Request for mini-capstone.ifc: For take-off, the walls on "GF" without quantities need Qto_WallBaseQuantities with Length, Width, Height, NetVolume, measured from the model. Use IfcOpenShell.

First a look at what the model holds.

```python
import ifcopenshell
import ifcopenshell.util.element
import ifcopenshell.util.unit

model = ifcopenshell.open("mini-capstone.ifc")
print(model.schema)
for unit_type in ("LENGTHUNIT", "AREAUNIT", "VOLUMEUNIT"):
    print(unit_type, ifcopenshell.util.unit.calculate_unit_scale(model, unit_type))
storey = next(s for s in model.by_type("IfcBuildingStorey") if s.Name == "GF")
walls = [e for e in ifcopenshell.util.element.get_decomposition(storey) if e.is_a("IfcWall")]
for e in sorted(walls, key=lambda e: e.id()):
    print(e.id(), e.is_a(), e.Name, list(ifcopenshell.util.element.get_psets(e, qtos_only=True)), sep=" | ")
```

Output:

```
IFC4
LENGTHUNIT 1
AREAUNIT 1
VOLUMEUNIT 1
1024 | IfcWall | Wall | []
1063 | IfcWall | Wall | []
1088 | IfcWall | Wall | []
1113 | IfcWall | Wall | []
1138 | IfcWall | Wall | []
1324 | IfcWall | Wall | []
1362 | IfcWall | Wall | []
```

```python
import ifcopenshell
import ifcopenshell.api.pset
import ifcopenshell.geom
import ifcopenshell.util.element
import ifcopenshell.util.shape
import ifcopenshell.util.unit

model = ifcopenshell.open("mini-capstone.ifc")
unit_scale = ifcopenshell.util.unit.calculate_unit_scale(model)
volume_scale = ifcopenshell.util.unit.calculate_unit_scale(model, "VOLUMEUNIT")
settings = ifcopenshell.geom.settings()

storey = next(s for s in model.by_type("IfcBuildingStorey") if s.Name == "GF")
walls = [e for e in ifcopenshell.util.element.get_decomposition(storey) if e.is_a("IfcWall")]

for e in sorted(walls, key=lambda e: e.id()):
    if ifcopenshell.util.element.get_psets(e, qtos_only=True, should_inherit=False):
        continue
    # Geometry comes back in metres, in the element's own axes.
    shape = ifcopenshell.geom.create_shape(settings, e)
    values = {
        "Length": ifcopenshell.util.shape.get_x(shape.geometry) / unit_scale,
        "Width": ifcopenshell.util.shape.get_y(shape.geometry) / unit_scale,
        "Height": ifcopenshell.util.shape.get_z(shape.geometry) / unit_scale,
        "NetVolume": ifcopenshell.util.shape.get_volume(shape.geometry) / volume_scale,
    }
    qto = ifcopenshell.api.pset.add_qto(model, product=e, name="Qto_WallBaseQuantities")
    ifcopenshell.api.pset.edit_qto(model, qto=qto, properties=values)
    print(e.id(), {k: round(v, 3) for k, v in values.items()})

model.write("mini-capstone-out.ifc")
```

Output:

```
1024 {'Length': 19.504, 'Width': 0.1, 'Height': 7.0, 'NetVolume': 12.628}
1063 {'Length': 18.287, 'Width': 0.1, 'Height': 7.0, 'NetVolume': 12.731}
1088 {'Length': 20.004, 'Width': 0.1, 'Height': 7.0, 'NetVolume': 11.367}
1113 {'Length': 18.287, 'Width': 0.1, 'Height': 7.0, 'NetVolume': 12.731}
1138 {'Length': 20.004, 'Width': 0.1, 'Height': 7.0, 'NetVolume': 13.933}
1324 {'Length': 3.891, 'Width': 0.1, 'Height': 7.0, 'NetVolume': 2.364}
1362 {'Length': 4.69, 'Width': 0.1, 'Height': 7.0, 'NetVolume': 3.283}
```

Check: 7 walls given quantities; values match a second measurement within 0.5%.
